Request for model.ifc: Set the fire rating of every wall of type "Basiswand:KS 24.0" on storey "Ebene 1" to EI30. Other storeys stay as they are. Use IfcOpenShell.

First a look at what the model holds.

```python
import ifcopenshell
import ifcopenshell.util.element

model = ifcopenshell.open("model.ifc")
print(model.schema)
storey = next(s for s in model.by_type("IfcBuildingStorey") if s.Name == "Ebene 1")
walls = [e for e in ifcopenshell.util.element.get_decomposition(storey) if e.is_a("IfcWall")]
seen = {}
for e in walls:
    element_type = ifcopenshell.util.element.get_type(e)
    key = (element_type.Name if element_type != e and element_type else None, ifcopenshell.util.element.get_pset(e, "Pset_WallCommon", "FireRating"))
    seen[key] = seen.get(key, 0) + 1
for (name, value), count in sorted(seen.items(), key=str):
    print(count, "x", name, "|", value)
```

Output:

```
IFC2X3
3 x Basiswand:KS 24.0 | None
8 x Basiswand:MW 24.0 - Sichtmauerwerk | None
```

```python
import ifcopenshell
import ifcopenshell.api.pset
import ifcopenshell.util.element

model = ifcopenshell.open("model.ifc")

storey = next(s for s in model.by_type("IfcBuildingStorey") if s.Name == "Ebene 1")
walls = [e for e in ifcopenshell.util.element.get_decomposition(storey) if e.is_a("IfcWall")]

count = 0
for e in walls:
    element_type = ifcopenshell.util.element.get_type(e)
    if element_type in (None, e) or element_type.Name != "Basiswand:KS 24.0":
        continue
    # add_pset returns the element's existing set when there is one.
    pset = ifcopenshell.api.pset.add_pset(model, product=e, name="Pset_WallCommon")
    ifcopenshell.api.pset.edit_pset(model, pset=pset, properties={"FireRating": "EI30"})
    count += 1

print(count, "walls updated")

model.write("model-out.ifc")
```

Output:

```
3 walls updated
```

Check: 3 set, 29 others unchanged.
